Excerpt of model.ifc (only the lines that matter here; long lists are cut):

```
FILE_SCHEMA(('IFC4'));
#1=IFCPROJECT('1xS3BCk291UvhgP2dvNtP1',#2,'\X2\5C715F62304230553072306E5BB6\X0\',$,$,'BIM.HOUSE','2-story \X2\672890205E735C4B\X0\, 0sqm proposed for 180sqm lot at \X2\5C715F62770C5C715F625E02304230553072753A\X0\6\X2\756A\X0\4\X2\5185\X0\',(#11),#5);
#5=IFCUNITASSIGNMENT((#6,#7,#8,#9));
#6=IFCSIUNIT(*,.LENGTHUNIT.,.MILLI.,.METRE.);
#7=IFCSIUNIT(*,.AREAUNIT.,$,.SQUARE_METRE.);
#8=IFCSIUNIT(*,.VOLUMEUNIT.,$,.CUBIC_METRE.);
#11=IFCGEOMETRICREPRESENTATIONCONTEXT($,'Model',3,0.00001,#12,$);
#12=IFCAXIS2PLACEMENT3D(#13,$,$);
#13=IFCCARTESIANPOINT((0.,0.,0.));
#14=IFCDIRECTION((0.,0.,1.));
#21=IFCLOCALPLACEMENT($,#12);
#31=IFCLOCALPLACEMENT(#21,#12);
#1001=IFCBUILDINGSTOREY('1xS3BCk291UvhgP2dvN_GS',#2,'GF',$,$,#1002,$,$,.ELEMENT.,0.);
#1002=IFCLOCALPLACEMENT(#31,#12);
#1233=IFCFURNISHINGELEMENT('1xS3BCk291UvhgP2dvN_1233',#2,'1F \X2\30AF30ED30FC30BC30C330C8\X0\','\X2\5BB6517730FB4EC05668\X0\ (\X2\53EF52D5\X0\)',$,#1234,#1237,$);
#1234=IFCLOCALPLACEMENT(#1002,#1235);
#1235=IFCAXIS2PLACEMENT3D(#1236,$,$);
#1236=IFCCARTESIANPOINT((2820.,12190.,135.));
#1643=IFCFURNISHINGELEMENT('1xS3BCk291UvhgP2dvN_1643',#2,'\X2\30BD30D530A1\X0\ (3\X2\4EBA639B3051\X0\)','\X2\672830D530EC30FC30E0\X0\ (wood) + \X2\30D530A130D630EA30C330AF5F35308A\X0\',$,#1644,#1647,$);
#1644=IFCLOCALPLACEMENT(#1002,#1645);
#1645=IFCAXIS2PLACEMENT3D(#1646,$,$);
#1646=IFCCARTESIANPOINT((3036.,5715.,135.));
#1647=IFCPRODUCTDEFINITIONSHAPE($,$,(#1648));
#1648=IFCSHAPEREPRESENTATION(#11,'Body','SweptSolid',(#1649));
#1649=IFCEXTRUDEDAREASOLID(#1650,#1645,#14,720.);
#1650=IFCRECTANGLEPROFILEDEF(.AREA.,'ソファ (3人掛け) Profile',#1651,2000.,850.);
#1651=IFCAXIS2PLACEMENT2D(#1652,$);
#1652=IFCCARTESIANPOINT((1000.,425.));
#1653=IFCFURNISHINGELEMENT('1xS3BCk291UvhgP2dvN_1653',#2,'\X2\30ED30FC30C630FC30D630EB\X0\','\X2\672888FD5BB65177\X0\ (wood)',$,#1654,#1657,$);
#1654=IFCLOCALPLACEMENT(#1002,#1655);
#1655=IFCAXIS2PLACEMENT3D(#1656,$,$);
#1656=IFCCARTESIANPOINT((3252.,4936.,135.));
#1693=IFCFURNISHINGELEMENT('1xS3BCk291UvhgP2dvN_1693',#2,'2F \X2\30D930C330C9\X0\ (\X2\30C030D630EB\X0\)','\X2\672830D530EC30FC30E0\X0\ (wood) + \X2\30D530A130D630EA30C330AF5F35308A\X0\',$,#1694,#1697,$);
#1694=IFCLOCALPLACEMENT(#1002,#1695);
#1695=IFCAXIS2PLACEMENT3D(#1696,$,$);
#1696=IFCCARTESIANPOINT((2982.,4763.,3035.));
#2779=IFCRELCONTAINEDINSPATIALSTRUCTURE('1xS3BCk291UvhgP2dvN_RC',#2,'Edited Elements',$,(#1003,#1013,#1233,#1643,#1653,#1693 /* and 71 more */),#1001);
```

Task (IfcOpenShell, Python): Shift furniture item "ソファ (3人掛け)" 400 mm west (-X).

```python
import ifcopenshell
import ifcopenshell.api.geometry
import ifcopenshell.util.placement
import ifcopenshell.util.unit

model = ifcopenshell.open("model.ifc")
unit_scale = ifcopenshell.util.unit.calculate_unit_scale(model)

item = model.by_guid("1xS3BCk291UvhgP2dvN_1643")
matrix = ifcopenshell.util.placement.get_local_placement(item.ObjectPlacement)
matrix[0, 3] -= 0.4 / unit_scale
ifcopenshell.api.geometry.edit_object_placement(model, product=item, matrix=matrix, is_si=False)

print(ifcopenshell.util.placement.get_local_placement(item.ObjectPlacement).round(3) + 0.0)

model.write("model_v2.ifc")
```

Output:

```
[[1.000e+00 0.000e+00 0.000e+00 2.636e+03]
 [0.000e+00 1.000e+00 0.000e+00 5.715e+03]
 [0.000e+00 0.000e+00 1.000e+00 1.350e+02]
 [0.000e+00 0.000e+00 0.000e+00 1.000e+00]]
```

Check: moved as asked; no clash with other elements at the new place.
